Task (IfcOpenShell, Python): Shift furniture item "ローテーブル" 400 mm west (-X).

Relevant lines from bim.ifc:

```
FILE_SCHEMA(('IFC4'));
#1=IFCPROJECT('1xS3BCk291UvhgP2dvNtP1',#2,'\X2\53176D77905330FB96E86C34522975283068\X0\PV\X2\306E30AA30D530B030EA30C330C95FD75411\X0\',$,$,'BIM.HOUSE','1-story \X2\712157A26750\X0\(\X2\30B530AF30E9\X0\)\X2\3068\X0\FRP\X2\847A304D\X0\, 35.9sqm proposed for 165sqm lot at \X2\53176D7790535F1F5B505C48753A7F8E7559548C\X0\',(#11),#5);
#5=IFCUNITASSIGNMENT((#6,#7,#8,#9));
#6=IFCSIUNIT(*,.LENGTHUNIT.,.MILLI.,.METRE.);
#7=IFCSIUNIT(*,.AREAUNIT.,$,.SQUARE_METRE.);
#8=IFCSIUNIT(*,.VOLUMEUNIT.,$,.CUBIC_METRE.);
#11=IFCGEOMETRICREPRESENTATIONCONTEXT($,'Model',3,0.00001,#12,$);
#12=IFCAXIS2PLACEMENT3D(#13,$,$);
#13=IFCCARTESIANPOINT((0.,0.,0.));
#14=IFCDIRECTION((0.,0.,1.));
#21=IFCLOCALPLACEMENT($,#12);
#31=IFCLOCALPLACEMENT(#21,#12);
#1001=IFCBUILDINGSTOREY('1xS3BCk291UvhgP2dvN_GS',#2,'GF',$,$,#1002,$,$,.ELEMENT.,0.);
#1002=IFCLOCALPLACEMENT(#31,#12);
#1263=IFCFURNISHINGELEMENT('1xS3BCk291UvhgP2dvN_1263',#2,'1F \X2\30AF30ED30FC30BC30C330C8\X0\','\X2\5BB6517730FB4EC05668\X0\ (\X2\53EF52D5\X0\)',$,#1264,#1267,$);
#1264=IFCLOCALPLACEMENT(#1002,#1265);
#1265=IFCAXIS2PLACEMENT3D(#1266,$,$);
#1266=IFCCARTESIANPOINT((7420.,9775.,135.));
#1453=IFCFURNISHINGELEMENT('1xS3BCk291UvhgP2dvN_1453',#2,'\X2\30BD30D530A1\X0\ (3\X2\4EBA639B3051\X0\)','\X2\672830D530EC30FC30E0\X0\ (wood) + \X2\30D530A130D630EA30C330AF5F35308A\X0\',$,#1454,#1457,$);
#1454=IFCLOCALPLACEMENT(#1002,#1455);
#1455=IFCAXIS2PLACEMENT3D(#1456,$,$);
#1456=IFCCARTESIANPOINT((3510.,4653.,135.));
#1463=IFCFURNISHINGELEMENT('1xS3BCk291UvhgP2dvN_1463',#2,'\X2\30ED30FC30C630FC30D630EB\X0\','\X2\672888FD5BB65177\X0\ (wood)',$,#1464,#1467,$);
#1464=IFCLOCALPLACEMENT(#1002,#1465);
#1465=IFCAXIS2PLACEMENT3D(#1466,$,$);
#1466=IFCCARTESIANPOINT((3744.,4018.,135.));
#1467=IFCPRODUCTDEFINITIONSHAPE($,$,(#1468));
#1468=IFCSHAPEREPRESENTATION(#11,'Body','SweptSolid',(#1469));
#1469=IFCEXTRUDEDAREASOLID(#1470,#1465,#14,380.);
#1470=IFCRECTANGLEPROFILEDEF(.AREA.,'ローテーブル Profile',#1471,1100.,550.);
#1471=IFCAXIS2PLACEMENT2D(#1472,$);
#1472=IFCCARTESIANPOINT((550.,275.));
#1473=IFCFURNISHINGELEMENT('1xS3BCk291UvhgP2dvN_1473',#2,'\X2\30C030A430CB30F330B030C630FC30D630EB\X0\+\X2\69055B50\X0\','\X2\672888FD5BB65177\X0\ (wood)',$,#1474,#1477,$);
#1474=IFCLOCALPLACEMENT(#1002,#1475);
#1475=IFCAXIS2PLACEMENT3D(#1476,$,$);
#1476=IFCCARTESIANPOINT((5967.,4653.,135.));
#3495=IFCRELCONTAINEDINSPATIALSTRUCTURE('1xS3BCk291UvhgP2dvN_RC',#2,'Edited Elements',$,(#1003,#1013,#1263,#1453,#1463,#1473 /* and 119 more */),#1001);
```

```python
import ifcopenshell
import ifcopenshell.api.geometry
import ifcopenshell.util.placement

model = ifcopenshell.open("bim.ifc")

item = model.by_guid("1xS3BCk291UvhgP2dvN_1463")
matrix = ifcopenshell.util.placement.get_local_placement(item.ObjectPlacement)
matrix[0, 3] -= 400.0
ifcopenshell.api.geometry.edit_object_placement(model, product=item, matrix=matrix, is_si=False)

print(ifcopenshell.util.placement.get_local_placement(item.ObjectPlacement).round(3) + 0.0)

model.write("bim_edited.ifc")
```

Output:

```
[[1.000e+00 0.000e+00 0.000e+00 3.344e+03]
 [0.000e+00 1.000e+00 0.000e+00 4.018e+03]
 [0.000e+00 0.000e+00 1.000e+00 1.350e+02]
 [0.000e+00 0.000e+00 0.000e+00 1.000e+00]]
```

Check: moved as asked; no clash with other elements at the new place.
